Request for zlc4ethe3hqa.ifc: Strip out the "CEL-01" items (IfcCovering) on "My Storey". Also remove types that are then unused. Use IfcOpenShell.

First a look at what the model holds.

```python
import ifcopenshell
import ifcopenshell.util.element

model = ifcopenshell.open("zlc4ethe3hqa.ifc")
print(model.schema)
storey = next(s for s in model.by_type("IfcBuildingStorey") if s.Name == "My Storey")
coverings = [e for e in ifcopenshell.util.element.get_decomposition(storey) if e.is_a("IfcCovering")]
seen = {}
for e in coverings:
    element_type = ifcopenshell.util.element.get_type(e)
    name = element_type.Name if element_type not in (None, e) else None
    seen[name] = seen.get(name, 0) + 1
for name, count in sorted(seen.items(), key=str):
    print(count, "x", name)
```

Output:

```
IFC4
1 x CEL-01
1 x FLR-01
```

```python
import ifcopenshell
import ifcopenshell.api.root
import ifcopenshell.util.element

model = ifcopenshell.open("zlc4ethe3hqa.ifc")

storey = next(s for s in model.by_type("IfcBuildingStorey") if s.Name == "My Storey")
coverings = [e for e in ifcopenshell.util.element.get_decomposition(storey) if e.is_a("IfcCovering")]
targets = [e for e in coverings if (t := ifcopenshell.util.element.get_type(e)) not in (None, e) and t.Name == "CEL-01"]
types = {ifcopenshell.util.element.get_type(e) for e in targets} - {None, *targets}

for e in targets:
    ifcopenshell.api.root.remove_product(model, product=e)
print(len(targets), "removed")

unused = [t for t in types if not ifcopenshell.util.element.get_types(t)]
for t in unused:
    ifcopenshell.api.root.remove_product(model, product=t)
print(len(unused), "unused types removed")

model.write("zlc4ethe3hqa_updated.ifc")
```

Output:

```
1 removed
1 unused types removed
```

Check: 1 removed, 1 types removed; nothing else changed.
